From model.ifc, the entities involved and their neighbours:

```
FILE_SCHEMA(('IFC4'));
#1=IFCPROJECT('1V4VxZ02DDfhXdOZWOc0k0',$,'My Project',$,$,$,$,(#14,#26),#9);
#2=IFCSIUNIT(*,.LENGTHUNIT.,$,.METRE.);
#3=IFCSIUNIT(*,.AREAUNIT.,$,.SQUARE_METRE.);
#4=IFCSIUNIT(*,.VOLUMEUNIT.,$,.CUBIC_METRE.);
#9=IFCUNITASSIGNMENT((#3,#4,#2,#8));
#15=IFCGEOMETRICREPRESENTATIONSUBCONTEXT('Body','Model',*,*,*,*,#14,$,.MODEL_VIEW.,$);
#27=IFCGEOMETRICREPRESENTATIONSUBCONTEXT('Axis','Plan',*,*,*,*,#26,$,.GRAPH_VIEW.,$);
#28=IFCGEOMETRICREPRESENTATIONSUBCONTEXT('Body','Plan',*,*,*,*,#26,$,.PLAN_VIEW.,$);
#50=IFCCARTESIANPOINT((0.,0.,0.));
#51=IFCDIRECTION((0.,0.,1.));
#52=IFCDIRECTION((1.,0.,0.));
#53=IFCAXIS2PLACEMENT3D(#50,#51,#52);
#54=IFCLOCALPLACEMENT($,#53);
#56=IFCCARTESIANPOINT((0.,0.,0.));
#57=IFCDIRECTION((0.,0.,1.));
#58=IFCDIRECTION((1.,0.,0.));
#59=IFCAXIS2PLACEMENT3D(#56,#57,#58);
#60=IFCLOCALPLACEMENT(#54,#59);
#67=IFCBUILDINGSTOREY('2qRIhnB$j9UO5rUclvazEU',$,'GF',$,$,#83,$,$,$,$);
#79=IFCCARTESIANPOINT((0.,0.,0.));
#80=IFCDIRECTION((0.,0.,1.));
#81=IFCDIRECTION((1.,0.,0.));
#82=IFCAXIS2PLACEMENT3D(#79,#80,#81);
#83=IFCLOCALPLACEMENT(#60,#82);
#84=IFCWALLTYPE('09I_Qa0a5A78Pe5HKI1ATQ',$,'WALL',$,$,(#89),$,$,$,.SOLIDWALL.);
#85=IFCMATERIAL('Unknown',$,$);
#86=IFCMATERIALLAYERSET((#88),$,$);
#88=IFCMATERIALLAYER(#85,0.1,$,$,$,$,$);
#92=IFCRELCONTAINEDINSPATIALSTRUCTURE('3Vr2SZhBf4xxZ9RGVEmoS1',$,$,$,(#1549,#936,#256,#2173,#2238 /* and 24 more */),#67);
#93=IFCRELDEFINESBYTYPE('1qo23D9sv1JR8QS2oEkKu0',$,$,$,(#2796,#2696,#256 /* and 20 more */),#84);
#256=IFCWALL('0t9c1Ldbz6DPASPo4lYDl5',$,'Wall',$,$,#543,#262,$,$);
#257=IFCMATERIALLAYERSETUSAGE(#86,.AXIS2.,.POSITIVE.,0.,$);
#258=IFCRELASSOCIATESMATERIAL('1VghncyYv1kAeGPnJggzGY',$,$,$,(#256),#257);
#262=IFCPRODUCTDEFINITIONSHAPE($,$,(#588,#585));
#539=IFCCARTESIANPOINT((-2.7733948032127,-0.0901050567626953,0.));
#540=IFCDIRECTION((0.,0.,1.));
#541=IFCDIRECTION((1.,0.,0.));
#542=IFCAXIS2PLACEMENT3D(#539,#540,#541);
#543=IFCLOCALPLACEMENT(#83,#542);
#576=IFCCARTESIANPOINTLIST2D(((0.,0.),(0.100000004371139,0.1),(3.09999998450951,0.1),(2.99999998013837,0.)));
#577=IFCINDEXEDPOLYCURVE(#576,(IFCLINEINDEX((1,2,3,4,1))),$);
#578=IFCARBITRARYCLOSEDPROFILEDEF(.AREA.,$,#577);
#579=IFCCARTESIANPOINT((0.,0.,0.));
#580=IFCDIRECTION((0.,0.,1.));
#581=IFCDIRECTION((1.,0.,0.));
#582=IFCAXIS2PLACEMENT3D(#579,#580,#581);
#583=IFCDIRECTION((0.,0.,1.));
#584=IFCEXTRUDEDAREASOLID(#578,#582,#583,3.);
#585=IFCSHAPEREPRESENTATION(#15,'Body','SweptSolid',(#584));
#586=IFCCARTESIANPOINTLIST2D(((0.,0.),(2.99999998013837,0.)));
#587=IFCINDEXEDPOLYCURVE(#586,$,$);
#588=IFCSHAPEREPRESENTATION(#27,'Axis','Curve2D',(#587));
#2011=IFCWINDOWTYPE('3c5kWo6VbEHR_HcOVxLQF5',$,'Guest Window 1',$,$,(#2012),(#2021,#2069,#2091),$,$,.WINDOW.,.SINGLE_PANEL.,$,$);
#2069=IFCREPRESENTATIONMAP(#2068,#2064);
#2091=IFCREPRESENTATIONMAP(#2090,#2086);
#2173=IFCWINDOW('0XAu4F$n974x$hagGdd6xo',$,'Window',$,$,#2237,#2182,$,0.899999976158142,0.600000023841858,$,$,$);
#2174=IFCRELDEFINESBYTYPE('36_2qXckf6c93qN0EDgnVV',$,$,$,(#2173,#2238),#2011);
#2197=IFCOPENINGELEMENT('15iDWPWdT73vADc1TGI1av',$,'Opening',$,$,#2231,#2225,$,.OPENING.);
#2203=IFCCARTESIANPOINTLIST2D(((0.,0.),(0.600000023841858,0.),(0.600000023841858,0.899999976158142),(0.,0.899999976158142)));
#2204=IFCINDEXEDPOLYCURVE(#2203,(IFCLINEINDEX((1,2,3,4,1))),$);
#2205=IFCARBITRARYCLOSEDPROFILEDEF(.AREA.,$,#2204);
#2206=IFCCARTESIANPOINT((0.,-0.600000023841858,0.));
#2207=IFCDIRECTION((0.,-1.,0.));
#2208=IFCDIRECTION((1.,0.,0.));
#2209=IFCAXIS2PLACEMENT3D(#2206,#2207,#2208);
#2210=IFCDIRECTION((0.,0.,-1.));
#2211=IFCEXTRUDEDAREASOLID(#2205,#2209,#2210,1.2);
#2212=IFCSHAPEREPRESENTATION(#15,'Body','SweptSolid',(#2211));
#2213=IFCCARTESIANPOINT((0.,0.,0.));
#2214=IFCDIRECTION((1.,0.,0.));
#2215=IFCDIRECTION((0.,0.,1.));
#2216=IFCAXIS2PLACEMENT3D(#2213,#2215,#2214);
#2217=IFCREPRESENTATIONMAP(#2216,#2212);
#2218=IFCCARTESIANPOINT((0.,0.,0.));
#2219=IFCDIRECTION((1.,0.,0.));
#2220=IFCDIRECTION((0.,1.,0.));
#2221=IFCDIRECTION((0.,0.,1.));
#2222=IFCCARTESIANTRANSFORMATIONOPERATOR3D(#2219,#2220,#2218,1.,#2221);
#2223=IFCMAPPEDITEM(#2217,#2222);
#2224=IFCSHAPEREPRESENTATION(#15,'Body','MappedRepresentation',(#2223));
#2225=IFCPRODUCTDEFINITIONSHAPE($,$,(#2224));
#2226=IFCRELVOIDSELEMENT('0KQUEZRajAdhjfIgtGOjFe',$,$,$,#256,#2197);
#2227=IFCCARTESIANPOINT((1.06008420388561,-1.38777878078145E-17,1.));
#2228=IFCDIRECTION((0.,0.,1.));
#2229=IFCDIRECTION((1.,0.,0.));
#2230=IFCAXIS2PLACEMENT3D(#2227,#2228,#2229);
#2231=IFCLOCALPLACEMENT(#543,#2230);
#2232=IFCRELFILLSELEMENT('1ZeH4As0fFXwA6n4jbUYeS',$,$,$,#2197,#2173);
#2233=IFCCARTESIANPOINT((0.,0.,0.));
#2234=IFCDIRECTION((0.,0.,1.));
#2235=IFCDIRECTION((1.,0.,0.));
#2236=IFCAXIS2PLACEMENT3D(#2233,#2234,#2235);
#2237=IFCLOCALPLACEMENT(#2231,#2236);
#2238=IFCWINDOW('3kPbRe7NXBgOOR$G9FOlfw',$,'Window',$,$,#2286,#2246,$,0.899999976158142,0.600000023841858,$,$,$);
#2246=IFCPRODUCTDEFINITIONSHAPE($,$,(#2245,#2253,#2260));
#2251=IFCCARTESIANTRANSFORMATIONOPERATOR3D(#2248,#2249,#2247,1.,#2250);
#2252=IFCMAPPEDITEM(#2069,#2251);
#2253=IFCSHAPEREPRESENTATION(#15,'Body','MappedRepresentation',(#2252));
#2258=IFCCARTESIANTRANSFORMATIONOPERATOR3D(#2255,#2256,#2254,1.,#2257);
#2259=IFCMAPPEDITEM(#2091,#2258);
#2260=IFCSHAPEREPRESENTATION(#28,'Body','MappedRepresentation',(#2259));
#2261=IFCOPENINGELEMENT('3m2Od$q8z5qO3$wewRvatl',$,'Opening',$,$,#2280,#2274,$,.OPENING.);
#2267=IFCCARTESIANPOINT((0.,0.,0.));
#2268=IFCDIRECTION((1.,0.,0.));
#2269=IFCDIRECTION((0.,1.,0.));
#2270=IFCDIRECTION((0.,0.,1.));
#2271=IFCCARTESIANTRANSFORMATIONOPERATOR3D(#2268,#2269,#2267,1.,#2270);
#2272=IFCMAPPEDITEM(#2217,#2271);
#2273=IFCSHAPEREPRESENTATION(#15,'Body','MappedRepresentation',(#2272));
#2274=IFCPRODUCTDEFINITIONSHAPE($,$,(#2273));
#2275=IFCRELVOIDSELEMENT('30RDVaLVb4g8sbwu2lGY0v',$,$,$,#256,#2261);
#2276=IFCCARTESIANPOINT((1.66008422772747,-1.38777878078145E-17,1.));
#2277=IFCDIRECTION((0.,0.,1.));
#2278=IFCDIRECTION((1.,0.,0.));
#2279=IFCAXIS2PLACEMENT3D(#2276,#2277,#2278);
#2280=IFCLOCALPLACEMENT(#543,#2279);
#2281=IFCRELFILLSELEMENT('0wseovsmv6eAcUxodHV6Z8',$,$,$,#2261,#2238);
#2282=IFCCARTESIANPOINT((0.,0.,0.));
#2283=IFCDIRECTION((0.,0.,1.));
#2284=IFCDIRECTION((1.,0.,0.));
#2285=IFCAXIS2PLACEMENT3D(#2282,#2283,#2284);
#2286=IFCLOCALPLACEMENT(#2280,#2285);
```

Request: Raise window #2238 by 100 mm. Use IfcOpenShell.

```python
import numpy as np
import ifcopenshell
import ifcopenshell.api.geometry
import ifcopenshell.util.placement
import ifcopenshell.util.unit

model = ifcopenshell.open("model.ifc")
unit_scale = ifcopenshell.util.unit.calculate_unit_scale(model)

window = model.by_guid("3kPbRe7NXBgOOR$G9FOlfw")
opening = window.FillsVoids[0].RelatingOpeningElement
dz = 0.1 / unit_scale

shift = np.array([0.0, 0.0, dz])
# The window is placed relative to its opening, so it follows when the opening moves.
matrix = ifcopenshell.util.placement.get_local_placement(opening.ObjectPlacement)
matrix[:3, 3] += shift
ifcopenshell.api.geometry.edit_object_placement(
    model, product=opening, matrix=matrix, is_si=False, should_transform_children=True
)

print(f"moved by {dz * unit_scale:+.3f} m")

model.write("model-out.ifc")
```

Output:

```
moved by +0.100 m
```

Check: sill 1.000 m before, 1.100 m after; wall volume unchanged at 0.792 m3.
